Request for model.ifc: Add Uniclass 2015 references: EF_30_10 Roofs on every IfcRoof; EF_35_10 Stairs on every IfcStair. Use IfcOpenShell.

First a look at what the model holds.

```python
import ifcopenshell

model = ifcopenshell.open("model.ifc")
print(model.schema)
print("classifications:", [c.Name for c in model.by_type("IfcClassification")])
for ifc_class in ("IfcDoor", "IfcRoof", "IfcStair", "IfcWall", "IfcWindow"):
    print(ifc_class, len(model.by_type(ifc_class)))
```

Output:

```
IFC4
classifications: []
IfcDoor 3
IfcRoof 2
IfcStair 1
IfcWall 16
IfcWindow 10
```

```python
import ifcopenshell
import ifcopenshell.api.classification

model = ifcopenshell.open("model.ifc")

system = ifcopenshell.api.classification.add_classification(model, classification="Uniclass 2015")

codes = {
    "IfcRoof": ("EF_30_10", "Roofs"),
    "IfcStair": ("EF_35_10", "Stairs"),
}
for ifc_class, (code, name) in codes.items():
    products = model.by_type(ifc_class)
    ifcopenshell.api.classification.add_reference(
        model, products=products, classification=system, identification=code, name=name
    )
    print(code, len(products))

model.write("model_v2.ifc")
```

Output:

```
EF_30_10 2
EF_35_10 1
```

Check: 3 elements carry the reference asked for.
